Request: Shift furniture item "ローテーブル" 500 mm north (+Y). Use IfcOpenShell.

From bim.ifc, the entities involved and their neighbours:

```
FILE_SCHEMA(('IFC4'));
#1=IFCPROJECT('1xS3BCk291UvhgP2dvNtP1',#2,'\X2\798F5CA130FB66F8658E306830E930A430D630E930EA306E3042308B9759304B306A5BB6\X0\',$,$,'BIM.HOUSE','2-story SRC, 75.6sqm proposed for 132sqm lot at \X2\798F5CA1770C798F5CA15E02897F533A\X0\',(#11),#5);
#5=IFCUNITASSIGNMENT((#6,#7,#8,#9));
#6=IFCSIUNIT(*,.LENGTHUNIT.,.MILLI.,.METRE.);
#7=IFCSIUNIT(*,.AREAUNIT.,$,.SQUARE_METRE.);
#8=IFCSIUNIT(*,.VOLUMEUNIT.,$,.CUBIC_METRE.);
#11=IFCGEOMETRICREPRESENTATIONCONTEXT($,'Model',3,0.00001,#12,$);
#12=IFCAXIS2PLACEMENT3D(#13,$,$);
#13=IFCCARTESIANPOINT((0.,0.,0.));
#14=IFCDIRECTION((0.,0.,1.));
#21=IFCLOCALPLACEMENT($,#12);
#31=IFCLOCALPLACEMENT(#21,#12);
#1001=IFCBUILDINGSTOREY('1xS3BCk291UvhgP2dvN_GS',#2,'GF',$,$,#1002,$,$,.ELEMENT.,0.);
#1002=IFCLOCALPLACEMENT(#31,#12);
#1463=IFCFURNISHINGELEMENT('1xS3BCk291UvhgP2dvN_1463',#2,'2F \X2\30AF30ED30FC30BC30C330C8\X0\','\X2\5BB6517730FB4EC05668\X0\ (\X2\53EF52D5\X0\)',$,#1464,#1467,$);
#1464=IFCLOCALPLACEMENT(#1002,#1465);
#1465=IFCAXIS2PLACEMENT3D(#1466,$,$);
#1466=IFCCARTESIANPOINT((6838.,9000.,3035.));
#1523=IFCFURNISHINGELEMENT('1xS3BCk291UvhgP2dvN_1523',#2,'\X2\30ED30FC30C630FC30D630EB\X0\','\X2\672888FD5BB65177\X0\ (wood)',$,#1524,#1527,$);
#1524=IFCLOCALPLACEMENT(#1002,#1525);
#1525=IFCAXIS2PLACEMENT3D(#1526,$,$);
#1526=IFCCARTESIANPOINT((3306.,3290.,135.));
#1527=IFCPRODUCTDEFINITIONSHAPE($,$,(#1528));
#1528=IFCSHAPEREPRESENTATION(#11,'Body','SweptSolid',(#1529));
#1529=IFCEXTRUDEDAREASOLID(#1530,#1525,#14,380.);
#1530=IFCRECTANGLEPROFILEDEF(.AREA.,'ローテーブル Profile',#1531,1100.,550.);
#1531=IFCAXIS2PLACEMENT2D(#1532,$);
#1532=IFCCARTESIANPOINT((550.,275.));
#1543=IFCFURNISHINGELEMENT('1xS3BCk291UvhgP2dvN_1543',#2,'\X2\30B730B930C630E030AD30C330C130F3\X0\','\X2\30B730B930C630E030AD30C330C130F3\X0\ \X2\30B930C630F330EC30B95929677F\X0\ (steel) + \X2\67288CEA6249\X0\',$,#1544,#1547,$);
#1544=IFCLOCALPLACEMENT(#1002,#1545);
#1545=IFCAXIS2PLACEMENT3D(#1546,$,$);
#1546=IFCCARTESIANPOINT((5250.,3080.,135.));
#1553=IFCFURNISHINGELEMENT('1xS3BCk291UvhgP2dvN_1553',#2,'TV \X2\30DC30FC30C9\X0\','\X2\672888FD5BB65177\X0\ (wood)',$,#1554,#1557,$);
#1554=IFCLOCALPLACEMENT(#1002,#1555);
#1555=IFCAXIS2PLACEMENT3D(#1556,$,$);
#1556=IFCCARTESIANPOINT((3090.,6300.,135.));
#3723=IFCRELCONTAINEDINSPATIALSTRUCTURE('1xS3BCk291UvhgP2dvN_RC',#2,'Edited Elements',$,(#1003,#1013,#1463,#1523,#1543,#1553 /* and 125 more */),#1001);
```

```python
import ifcopenshell
import ifcopenshell.api.geometry
import ifcopenshell.util.placement

model = ifcopenshell.open("bim.ifc")

item = model.by_id(1523)
matrix = ifcopenshell.util.placement.get_local_placement(item.ObjectPlacement)
matrix[1, 3] += 500.0
ifcopenshell.api.geometry.edit_object_placement(model, product=item, matrix=matrix, is_si=False)

print(ifcopenshell.util.placement.get_local_placement(item.ObjectPlacement).round(3) + 0.0)

model.write("bim_updated.ifc")
```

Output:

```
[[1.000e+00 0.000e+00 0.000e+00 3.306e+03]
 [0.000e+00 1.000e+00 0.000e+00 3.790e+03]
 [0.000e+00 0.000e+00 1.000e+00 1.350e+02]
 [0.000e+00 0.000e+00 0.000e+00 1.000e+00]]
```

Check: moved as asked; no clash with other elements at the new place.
